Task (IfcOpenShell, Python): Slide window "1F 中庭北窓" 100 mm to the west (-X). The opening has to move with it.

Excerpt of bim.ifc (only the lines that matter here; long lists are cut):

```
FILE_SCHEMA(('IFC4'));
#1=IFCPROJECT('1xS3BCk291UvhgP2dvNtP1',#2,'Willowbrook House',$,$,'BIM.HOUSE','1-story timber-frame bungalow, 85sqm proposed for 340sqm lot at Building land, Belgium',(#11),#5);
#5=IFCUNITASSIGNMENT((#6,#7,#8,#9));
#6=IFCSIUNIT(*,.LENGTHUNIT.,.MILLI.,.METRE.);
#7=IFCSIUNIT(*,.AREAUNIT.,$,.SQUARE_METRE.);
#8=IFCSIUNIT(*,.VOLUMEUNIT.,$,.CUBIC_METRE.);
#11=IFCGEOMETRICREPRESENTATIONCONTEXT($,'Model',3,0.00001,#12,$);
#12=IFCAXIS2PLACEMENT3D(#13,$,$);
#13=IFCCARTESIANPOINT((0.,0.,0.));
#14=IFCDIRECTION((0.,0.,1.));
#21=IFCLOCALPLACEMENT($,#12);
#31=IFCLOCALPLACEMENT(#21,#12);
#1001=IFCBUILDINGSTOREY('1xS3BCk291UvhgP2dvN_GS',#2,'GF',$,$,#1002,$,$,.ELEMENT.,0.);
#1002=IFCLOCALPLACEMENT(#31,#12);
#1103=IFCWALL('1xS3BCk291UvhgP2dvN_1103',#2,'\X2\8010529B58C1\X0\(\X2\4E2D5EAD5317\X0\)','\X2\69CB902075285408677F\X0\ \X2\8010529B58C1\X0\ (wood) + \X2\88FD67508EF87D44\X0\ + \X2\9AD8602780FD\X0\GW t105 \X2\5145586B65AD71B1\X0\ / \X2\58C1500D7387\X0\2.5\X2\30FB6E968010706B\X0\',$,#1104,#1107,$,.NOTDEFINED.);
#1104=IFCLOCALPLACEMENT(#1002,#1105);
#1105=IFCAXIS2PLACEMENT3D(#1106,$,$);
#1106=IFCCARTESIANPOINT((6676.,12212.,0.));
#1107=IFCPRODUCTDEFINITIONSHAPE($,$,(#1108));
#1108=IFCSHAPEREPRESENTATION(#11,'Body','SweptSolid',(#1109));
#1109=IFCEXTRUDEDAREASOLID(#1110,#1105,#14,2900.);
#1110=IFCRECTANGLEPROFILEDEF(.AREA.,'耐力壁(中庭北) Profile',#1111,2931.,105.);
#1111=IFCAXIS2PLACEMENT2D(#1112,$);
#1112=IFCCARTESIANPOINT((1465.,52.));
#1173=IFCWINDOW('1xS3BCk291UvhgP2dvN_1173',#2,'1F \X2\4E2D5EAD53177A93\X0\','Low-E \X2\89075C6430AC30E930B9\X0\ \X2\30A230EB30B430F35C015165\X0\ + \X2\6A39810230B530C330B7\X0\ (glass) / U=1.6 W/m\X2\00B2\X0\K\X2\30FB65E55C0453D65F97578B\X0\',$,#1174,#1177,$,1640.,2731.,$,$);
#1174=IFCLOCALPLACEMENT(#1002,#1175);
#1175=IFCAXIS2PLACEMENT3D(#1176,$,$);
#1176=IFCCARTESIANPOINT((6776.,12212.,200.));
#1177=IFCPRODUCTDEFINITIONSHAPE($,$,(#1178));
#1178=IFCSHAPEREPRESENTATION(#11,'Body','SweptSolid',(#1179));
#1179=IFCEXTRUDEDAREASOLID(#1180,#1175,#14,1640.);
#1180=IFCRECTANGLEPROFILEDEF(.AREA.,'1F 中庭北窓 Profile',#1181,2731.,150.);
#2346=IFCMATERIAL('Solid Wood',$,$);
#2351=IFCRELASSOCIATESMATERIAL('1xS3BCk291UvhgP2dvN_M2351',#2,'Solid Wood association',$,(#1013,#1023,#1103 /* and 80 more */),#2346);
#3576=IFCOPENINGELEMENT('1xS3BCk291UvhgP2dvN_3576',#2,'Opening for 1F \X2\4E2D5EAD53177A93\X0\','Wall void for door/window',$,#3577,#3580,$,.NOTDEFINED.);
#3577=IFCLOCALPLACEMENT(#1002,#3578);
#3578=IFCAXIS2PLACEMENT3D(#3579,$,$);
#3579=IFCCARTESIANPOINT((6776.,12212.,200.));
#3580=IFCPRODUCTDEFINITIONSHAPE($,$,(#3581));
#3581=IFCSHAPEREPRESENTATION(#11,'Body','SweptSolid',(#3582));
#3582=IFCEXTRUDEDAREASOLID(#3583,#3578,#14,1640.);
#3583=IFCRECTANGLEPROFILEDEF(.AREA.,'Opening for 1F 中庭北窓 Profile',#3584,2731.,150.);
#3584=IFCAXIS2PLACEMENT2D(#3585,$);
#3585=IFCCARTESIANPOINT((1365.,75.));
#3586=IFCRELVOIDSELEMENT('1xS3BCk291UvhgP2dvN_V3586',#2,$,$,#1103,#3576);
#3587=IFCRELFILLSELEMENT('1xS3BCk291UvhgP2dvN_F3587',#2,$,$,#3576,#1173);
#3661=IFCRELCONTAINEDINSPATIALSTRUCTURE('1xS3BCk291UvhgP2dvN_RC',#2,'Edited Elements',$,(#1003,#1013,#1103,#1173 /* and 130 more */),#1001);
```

```python
import ifcopenshell
import ifcopenshell.api.geometry
import ifcopenshell.util.placement
import ifcopenshell.util.unit

model = ifcopenshell.open("bim.ifc")
unit_scale = ifcopenshell.util.unit.calculate_unit_scale(model)

window = model.by_guid("1xS3BCk291UvhgP2dvN_1173")
opening = window.FillsVoids[0].RelatingOpeningElement
wall = opening.VoidsElements[0].RelatingBuildingElement

wall_matrix = ifcopenshell.util.placement.get_local_placement(wall.ObjectPlacement)
shift = wall_matrix[:3, 0] * -0.1 / unit_scale
before = ifcopenshell.util.placement.get_local_placement(window.ObjectPlacement)[:3, 3].copy()

# The window is not placed relative to its opening, so move both.
for product in (opening, window):
    matrix = ifcopenshell.util.placement.get_local_placement(product.ObjectPlacement)
    matrix[:3, 3] += shift
    ifcopenshell.api.geometry.edit_object_placement(model, product=product, matrix=matrix, is_si=False)

after = ifcopenshell.util.placement.get_local_placement(window.ObjectPlacement)[:3, 3]
print("window moved by", (after - before).round(3) + 0.0)

model.write("bim_updated.ifc")
```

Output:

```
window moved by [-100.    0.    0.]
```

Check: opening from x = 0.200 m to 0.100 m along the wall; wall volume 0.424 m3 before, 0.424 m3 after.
